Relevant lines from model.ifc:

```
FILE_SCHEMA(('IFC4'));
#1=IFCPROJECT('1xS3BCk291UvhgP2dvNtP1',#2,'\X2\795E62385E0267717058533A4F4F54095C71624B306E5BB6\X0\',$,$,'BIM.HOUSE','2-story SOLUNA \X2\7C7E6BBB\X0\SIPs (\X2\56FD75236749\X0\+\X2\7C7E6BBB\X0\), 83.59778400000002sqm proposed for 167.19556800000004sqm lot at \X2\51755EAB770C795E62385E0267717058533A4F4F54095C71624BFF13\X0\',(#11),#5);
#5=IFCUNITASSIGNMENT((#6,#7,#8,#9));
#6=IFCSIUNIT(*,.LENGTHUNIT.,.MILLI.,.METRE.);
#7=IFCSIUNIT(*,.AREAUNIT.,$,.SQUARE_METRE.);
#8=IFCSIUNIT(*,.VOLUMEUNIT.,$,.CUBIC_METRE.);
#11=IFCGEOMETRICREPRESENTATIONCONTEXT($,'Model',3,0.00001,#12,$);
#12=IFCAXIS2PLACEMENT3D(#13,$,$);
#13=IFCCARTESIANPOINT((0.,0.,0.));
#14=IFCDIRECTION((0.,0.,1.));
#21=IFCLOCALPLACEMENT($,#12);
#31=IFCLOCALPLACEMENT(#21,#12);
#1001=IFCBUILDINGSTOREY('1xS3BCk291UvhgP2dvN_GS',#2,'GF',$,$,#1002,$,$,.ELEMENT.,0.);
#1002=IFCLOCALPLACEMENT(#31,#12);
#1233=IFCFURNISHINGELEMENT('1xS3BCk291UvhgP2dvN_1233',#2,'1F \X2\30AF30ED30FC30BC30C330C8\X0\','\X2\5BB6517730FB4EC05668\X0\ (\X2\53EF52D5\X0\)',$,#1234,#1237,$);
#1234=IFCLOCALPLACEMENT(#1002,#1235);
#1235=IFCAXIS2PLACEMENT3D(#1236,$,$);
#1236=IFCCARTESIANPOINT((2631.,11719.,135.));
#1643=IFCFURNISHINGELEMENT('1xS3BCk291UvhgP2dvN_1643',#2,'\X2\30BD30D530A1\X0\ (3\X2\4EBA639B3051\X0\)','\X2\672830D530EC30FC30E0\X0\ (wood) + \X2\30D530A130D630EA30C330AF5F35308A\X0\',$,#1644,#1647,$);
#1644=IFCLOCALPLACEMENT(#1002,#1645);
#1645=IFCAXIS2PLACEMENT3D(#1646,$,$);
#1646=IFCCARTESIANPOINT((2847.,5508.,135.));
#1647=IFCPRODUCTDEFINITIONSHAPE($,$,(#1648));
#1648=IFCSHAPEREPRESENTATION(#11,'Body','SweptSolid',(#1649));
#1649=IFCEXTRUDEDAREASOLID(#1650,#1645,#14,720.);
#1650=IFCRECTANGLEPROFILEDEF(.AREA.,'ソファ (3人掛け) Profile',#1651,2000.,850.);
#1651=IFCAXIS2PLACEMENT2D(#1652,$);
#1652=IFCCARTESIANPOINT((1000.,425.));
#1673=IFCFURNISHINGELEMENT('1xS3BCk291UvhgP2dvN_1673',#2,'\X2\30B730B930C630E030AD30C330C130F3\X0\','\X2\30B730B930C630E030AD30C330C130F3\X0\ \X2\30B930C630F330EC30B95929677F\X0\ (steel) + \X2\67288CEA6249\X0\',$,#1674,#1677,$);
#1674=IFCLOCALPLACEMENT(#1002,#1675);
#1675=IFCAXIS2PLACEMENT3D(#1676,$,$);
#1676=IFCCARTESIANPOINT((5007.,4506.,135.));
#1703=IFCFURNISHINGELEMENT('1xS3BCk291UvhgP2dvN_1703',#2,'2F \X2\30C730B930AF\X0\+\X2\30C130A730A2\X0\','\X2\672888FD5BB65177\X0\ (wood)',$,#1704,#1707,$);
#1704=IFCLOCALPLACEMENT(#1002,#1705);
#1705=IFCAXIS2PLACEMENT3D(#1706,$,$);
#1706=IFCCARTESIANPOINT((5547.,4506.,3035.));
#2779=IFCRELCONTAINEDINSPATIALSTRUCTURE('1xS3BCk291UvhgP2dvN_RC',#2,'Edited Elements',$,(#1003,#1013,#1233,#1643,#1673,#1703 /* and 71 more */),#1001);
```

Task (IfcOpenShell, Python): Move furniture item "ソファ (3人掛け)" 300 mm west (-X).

```python
import ifcopenshell
import ifcopenshell.api.geometry
import ifcopenshell.util.placement
import ifcopenshell.util.unit

model = ifcopenshell.open("model.ifc")
unit_scale = ifcopenshell.util.unit.calculate_unit_scale(model)

item = model.by_guid("1xS3BCk291UvhgP2dvN_1643")
matrix = ifcopenshell.util.placement.get_local_placement(item.ObjectPlacement)
matrix[0, 3] -= 0.3 / unit_scale
ifcopenshell.api.geometry.edit_object_placement(model, product=item, matrix=matrix, is_si=False)

print(ifcopenshell.util.placement.get_local_placement(item.ObjectPlacement).round(3) + 0.0)

model.write("model_v2.ifc")
```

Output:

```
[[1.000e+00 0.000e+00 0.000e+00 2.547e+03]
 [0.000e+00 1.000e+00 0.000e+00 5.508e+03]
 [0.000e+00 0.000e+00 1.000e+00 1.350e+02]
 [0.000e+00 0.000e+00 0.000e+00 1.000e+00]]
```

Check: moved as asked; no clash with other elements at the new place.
